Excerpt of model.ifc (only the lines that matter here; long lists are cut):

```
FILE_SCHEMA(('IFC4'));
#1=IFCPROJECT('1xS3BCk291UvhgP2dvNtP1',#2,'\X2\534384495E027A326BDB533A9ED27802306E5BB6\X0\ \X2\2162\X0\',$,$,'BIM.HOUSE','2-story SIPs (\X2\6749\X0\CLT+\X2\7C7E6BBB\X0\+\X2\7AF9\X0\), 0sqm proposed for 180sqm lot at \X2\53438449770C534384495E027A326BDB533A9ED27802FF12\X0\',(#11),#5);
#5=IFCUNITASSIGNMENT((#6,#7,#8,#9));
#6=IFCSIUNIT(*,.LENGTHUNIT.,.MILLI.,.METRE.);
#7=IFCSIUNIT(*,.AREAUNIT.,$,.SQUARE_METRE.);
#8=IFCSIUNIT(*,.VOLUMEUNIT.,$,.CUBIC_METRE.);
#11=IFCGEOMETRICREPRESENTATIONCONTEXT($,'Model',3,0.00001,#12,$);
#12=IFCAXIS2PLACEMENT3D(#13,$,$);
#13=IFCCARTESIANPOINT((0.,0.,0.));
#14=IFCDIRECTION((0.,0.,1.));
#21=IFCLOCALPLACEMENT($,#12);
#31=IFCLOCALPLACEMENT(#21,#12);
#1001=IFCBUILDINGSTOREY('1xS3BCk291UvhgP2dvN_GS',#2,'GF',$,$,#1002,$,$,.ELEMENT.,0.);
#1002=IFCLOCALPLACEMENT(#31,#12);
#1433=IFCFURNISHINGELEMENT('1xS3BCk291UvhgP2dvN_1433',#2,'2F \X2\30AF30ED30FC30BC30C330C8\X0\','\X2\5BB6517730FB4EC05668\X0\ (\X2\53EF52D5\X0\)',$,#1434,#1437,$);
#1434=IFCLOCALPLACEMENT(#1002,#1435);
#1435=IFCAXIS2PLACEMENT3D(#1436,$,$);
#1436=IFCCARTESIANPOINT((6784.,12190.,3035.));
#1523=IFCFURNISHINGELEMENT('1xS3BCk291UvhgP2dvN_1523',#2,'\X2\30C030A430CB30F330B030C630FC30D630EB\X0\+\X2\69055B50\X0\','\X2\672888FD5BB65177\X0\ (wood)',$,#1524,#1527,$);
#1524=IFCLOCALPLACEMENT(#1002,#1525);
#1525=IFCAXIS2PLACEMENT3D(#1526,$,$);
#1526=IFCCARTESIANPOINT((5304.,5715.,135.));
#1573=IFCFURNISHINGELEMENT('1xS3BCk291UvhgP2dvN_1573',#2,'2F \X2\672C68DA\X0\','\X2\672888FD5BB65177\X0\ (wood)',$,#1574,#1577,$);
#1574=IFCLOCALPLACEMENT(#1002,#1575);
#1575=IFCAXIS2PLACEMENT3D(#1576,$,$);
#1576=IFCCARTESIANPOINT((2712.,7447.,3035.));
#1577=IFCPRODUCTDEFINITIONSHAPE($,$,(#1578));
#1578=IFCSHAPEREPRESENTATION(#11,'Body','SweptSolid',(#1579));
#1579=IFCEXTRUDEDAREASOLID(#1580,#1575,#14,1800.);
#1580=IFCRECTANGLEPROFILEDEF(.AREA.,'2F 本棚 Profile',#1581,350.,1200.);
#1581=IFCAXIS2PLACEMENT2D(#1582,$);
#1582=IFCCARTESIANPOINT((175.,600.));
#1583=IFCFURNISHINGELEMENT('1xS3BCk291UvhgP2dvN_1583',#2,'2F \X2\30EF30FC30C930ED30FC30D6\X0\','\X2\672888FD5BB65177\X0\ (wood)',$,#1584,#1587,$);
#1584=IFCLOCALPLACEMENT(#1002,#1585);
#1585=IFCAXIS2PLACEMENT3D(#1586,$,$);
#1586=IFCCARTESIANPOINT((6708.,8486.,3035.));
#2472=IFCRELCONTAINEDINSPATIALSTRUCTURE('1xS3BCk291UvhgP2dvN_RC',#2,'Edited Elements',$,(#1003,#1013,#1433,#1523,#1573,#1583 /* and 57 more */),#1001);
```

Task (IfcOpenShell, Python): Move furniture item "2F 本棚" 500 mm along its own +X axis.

```python
import ifcopenshell
import ifcopenshell.api.geometry
import ifcopenshell.util.placement
import ifcopenshell.util.unit

model = ifcopenshell.open("model.ifc")
unit_scale = ifcopenshell.util.unit.calculate_unit_scale(model)

item = model.by_guid("1xS3BCk291UvhgP2dvN_1573")
matrix = ifcopenshell.util.placement.get_local_placement(item.ObjectPlacement)
matrix[:3, 3] += matrix[:3, 0] * 0.5 / unit_scale
ifcopenshell.api.geometry.edit_object_placement(model, product=item, matrix=matrix, is_si=False)

print(ifcopenshell.util.placement.get_local_placement(item.ObjectPlacement).round(3) + 0.0)

model.write("model-out.ifc")
```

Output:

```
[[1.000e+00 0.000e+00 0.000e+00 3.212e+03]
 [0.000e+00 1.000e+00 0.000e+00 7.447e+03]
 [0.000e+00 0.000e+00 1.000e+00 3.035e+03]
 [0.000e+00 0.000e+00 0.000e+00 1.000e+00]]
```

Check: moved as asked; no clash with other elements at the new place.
